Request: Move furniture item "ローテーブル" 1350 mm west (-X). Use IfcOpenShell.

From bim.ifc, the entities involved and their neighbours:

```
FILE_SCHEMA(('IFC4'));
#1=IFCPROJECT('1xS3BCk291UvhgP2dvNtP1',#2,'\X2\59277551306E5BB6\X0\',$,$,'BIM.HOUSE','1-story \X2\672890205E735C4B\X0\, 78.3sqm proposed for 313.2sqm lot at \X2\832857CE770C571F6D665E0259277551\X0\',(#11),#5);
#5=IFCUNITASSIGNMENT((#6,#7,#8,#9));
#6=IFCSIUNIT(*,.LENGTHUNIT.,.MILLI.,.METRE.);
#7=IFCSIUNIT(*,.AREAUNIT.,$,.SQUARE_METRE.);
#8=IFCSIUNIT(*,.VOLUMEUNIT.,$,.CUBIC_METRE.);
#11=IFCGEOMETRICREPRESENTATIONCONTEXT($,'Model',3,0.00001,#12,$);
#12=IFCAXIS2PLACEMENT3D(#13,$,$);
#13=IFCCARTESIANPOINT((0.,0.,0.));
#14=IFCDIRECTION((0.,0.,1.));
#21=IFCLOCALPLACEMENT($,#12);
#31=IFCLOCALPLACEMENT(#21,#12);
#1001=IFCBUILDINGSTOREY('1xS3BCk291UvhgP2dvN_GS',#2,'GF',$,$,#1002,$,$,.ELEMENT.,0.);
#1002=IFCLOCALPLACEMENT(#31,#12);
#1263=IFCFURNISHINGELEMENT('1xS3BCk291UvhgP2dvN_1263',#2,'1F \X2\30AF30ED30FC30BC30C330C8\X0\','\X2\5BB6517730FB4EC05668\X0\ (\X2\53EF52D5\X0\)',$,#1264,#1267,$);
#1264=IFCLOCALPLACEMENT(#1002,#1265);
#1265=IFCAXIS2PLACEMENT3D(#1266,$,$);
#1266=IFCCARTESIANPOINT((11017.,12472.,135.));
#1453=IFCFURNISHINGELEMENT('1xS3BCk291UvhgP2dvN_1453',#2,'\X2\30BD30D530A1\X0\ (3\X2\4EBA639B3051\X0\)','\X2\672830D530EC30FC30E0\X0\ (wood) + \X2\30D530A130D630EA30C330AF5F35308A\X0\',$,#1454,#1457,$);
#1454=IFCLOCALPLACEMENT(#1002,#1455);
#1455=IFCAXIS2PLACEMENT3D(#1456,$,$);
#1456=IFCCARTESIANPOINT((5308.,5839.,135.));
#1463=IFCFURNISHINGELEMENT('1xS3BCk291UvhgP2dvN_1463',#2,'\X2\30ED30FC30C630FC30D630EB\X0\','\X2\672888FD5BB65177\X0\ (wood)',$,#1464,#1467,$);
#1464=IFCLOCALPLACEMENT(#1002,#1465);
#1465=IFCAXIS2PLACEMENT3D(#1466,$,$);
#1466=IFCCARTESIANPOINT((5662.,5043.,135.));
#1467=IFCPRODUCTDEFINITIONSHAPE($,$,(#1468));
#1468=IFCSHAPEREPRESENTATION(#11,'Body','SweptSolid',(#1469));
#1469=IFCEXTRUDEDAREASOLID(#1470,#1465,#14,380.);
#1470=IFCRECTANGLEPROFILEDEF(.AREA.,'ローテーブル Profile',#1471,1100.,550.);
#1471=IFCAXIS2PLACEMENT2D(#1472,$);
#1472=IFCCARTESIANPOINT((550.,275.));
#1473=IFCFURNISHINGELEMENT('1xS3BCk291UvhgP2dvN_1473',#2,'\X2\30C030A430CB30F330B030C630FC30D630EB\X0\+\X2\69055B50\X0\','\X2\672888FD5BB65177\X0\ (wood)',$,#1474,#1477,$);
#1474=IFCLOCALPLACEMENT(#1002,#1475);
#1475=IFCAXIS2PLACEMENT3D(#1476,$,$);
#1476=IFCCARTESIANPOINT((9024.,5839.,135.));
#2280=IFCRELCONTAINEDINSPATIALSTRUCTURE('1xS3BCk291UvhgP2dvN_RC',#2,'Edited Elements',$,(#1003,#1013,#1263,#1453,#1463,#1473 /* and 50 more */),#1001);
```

```python
import ifcopenshell
import ifcopenshell.api.geometry
import ifcopenshell.util.placement

model = ifcopenshell.open("bim.ifc")

item = model.by_guid("1xS3BCk291UvhgP2dvN_1463")
matrix = ifcopenshell.util.placement.get_local_placement(item.ObjectPlacement)
matrix[0, 3] -= 1350.0
ifcopenshell.api.geometry.edit_object_placement(model, product=item, matrix=matrix, is_si=False)

print(ifcopenshell.util.placement.get_local_placement(item.ObjectPlacement).round(3) + 0.0)

model.write("bim-out.ifc")
```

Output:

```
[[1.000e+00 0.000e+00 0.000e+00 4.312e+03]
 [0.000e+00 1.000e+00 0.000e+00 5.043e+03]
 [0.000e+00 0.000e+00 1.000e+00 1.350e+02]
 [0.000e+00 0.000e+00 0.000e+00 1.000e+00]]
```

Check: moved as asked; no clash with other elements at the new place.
